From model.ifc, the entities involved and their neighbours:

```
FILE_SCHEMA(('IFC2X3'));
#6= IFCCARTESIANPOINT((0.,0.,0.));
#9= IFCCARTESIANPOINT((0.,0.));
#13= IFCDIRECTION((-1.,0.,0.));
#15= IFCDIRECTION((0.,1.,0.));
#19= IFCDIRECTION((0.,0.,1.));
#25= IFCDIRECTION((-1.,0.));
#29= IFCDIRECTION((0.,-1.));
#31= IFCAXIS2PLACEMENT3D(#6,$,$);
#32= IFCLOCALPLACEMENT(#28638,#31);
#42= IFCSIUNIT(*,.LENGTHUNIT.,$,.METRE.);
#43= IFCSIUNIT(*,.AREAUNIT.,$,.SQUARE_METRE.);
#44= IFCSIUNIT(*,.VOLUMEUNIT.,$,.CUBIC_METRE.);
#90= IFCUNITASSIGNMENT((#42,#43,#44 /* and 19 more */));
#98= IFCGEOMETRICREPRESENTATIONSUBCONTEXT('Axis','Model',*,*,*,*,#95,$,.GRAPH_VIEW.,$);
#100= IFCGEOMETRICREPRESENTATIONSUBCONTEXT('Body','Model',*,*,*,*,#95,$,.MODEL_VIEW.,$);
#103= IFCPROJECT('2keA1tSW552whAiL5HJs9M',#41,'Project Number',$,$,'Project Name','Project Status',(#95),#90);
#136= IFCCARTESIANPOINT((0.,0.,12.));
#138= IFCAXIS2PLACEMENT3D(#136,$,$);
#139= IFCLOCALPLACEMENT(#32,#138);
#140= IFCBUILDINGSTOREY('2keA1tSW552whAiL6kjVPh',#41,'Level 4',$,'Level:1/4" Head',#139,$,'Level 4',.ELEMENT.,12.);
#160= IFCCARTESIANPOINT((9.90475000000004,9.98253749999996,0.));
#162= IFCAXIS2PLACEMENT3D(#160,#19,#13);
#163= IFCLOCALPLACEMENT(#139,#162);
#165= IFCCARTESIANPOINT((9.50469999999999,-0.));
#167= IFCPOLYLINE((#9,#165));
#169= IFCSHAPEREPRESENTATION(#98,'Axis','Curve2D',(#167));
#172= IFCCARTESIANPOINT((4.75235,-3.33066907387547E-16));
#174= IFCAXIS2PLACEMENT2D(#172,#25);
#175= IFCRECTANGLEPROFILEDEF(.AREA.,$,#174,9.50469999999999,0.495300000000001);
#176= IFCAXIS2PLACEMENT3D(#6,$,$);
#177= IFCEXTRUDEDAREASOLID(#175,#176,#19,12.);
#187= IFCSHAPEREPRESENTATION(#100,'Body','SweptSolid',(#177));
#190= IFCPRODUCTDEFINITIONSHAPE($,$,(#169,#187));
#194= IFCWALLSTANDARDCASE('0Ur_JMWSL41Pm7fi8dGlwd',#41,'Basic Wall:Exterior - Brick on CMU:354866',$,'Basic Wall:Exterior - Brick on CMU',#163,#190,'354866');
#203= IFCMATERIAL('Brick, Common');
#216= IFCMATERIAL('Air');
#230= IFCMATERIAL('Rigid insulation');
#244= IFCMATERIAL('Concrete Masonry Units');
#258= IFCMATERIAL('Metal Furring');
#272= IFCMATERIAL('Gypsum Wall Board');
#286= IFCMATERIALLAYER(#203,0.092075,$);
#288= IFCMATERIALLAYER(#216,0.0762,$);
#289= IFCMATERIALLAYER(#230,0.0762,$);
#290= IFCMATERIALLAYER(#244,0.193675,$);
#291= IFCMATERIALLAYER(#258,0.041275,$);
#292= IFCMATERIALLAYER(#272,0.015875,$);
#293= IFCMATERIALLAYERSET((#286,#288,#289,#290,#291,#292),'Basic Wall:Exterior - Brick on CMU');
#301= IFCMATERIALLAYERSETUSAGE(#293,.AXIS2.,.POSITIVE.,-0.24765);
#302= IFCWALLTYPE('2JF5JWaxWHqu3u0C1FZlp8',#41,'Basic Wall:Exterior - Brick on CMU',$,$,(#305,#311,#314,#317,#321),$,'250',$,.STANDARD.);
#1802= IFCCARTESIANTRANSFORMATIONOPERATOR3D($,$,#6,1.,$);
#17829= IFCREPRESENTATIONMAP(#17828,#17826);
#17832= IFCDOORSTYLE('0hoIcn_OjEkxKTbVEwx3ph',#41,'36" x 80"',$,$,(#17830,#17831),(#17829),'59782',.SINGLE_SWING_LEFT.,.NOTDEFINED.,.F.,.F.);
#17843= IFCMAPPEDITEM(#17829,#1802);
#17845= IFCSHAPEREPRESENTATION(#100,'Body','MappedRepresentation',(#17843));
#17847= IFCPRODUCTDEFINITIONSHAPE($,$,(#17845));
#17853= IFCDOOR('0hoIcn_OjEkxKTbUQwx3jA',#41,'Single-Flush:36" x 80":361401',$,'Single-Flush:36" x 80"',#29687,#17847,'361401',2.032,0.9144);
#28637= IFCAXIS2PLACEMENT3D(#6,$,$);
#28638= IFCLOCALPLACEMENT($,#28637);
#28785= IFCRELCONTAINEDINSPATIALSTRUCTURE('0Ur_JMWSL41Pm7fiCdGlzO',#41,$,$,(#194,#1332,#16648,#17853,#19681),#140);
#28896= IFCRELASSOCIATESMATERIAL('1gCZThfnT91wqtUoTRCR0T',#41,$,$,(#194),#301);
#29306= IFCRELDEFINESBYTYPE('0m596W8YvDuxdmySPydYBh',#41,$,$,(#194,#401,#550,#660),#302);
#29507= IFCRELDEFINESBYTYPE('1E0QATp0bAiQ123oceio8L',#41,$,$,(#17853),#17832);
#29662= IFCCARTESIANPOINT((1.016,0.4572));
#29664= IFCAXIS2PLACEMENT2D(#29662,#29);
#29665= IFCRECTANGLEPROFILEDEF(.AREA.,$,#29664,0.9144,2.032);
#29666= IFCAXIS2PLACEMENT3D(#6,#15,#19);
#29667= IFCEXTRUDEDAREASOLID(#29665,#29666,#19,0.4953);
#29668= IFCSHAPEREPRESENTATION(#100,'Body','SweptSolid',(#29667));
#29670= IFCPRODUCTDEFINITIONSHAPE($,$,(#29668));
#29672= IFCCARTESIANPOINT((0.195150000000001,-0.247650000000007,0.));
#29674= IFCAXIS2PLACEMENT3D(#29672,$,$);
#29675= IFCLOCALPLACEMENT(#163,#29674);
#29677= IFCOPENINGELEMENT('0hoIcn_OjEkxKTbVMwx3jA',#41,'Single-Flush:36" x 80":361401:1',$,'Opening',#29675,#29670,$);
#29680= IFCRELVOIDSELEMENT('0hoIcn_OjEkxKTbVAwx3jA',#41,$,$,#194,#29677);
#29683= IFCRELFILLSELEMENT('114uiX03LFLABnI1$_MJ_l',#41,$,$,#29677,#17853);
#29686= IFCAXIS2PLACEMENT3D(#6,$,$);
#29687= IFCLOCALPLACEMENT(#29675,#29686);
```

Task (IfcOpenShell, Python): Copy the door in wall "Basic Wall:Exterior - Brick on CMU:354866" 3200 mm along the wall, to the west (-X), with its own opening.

```python
import ifcopenshell
import ifcopenshell.api.feature
import ifcopenshell.api.geometry
import ifcopenshell.api.root
import ifcopenshell.geom
import ifcopenshell.util.element
import ifcopenshell.util.placement
import ifcopenshell.util.shape

model = ifcopenshell.open("model.ifc")
settings = ifcopenshell.geom.settings()


def volume(element):
    """Net volume in cubic metres, openings subtracted."""
    shape = ifcopenshell.geom.create_shape(settings, element)
    return ifcopenshell.util.shape.get_volume(shape.geometry)


def reuse_history(source, copy):
    """copy_class also copies each property set's owner history, people and application; keep the originals."""
    for rel in copy.IsDefinedBy:
        if rel.is_a("IfcRelDefinesByProperties") and (history := rel.RelatingPropertyDefinition.OwnerHistory):
            rel.RelatingPropertyDefinition.OwnerHistory = source.OwnerHistory
            ifcopenshell.util.element.remove_deep2(model, history)


door = model.by_id(17853)
opening = door.FillsVoids[0].RelatingOpeningElement
wall = opening.VoidsElements[0].RelatingBuildingElement
before = volume(wall)
shift = ifcopenshell.util.placement.get_local_placement(wall.ObjectPlacement)[:3, 0] * 3.2

# copy_class copies the void relationship, type, container and properties, but no geometry.
new_opening = ifcopenshell.api.root.copy_class(model, product=opening)
new_opening.Representation = ifcopenshell.util.element.copy_deep(
    model, opening.Representation, exclude=["IfcGeometricRepresentationContext", "IfcRepresentationMap"]
)
new_opening.Name = 'Single-Flush:36" x 80"'
new_door = ifcopenshell.api.root.copy_class(model, product=door)
new_door.Representation = ifcopenshell.util.element.copy_deep(
    model, door.Representation, exclude=["IfcGeometricRepresentationContext", "IfcRepresentationMap"]
)
new_door.Name = 'Single-Flush:36" x 80"'
new_door.Tag = None
reuse_history(door, new_door)
fills = ifcopenshell.api.feature.add_filling(model, opening=new_opening, element=new_door)
fills.OwnerHistory = new_door.OwnerHistory  # required in IFC2X3

for old, new in ((opening, new_opening), (door, new_door)):
    matrix = ifcopenshell.util.placement.get_local_placement(old.ObjectPlacement)
    matrix[:3, 3] += shift
    ifcopenshell.api.geometry.edit_object_placement(model, product=new, matrix=matrix, is_si=False)

after = volume(wall)

print(f"wall volume {before:.3f} -> {after:.3f} m3")

model.write("model_updated.ifc")
```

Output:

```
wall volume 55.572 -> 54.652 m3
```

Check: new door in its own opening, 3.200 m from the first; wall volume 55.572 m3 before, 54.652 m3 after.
